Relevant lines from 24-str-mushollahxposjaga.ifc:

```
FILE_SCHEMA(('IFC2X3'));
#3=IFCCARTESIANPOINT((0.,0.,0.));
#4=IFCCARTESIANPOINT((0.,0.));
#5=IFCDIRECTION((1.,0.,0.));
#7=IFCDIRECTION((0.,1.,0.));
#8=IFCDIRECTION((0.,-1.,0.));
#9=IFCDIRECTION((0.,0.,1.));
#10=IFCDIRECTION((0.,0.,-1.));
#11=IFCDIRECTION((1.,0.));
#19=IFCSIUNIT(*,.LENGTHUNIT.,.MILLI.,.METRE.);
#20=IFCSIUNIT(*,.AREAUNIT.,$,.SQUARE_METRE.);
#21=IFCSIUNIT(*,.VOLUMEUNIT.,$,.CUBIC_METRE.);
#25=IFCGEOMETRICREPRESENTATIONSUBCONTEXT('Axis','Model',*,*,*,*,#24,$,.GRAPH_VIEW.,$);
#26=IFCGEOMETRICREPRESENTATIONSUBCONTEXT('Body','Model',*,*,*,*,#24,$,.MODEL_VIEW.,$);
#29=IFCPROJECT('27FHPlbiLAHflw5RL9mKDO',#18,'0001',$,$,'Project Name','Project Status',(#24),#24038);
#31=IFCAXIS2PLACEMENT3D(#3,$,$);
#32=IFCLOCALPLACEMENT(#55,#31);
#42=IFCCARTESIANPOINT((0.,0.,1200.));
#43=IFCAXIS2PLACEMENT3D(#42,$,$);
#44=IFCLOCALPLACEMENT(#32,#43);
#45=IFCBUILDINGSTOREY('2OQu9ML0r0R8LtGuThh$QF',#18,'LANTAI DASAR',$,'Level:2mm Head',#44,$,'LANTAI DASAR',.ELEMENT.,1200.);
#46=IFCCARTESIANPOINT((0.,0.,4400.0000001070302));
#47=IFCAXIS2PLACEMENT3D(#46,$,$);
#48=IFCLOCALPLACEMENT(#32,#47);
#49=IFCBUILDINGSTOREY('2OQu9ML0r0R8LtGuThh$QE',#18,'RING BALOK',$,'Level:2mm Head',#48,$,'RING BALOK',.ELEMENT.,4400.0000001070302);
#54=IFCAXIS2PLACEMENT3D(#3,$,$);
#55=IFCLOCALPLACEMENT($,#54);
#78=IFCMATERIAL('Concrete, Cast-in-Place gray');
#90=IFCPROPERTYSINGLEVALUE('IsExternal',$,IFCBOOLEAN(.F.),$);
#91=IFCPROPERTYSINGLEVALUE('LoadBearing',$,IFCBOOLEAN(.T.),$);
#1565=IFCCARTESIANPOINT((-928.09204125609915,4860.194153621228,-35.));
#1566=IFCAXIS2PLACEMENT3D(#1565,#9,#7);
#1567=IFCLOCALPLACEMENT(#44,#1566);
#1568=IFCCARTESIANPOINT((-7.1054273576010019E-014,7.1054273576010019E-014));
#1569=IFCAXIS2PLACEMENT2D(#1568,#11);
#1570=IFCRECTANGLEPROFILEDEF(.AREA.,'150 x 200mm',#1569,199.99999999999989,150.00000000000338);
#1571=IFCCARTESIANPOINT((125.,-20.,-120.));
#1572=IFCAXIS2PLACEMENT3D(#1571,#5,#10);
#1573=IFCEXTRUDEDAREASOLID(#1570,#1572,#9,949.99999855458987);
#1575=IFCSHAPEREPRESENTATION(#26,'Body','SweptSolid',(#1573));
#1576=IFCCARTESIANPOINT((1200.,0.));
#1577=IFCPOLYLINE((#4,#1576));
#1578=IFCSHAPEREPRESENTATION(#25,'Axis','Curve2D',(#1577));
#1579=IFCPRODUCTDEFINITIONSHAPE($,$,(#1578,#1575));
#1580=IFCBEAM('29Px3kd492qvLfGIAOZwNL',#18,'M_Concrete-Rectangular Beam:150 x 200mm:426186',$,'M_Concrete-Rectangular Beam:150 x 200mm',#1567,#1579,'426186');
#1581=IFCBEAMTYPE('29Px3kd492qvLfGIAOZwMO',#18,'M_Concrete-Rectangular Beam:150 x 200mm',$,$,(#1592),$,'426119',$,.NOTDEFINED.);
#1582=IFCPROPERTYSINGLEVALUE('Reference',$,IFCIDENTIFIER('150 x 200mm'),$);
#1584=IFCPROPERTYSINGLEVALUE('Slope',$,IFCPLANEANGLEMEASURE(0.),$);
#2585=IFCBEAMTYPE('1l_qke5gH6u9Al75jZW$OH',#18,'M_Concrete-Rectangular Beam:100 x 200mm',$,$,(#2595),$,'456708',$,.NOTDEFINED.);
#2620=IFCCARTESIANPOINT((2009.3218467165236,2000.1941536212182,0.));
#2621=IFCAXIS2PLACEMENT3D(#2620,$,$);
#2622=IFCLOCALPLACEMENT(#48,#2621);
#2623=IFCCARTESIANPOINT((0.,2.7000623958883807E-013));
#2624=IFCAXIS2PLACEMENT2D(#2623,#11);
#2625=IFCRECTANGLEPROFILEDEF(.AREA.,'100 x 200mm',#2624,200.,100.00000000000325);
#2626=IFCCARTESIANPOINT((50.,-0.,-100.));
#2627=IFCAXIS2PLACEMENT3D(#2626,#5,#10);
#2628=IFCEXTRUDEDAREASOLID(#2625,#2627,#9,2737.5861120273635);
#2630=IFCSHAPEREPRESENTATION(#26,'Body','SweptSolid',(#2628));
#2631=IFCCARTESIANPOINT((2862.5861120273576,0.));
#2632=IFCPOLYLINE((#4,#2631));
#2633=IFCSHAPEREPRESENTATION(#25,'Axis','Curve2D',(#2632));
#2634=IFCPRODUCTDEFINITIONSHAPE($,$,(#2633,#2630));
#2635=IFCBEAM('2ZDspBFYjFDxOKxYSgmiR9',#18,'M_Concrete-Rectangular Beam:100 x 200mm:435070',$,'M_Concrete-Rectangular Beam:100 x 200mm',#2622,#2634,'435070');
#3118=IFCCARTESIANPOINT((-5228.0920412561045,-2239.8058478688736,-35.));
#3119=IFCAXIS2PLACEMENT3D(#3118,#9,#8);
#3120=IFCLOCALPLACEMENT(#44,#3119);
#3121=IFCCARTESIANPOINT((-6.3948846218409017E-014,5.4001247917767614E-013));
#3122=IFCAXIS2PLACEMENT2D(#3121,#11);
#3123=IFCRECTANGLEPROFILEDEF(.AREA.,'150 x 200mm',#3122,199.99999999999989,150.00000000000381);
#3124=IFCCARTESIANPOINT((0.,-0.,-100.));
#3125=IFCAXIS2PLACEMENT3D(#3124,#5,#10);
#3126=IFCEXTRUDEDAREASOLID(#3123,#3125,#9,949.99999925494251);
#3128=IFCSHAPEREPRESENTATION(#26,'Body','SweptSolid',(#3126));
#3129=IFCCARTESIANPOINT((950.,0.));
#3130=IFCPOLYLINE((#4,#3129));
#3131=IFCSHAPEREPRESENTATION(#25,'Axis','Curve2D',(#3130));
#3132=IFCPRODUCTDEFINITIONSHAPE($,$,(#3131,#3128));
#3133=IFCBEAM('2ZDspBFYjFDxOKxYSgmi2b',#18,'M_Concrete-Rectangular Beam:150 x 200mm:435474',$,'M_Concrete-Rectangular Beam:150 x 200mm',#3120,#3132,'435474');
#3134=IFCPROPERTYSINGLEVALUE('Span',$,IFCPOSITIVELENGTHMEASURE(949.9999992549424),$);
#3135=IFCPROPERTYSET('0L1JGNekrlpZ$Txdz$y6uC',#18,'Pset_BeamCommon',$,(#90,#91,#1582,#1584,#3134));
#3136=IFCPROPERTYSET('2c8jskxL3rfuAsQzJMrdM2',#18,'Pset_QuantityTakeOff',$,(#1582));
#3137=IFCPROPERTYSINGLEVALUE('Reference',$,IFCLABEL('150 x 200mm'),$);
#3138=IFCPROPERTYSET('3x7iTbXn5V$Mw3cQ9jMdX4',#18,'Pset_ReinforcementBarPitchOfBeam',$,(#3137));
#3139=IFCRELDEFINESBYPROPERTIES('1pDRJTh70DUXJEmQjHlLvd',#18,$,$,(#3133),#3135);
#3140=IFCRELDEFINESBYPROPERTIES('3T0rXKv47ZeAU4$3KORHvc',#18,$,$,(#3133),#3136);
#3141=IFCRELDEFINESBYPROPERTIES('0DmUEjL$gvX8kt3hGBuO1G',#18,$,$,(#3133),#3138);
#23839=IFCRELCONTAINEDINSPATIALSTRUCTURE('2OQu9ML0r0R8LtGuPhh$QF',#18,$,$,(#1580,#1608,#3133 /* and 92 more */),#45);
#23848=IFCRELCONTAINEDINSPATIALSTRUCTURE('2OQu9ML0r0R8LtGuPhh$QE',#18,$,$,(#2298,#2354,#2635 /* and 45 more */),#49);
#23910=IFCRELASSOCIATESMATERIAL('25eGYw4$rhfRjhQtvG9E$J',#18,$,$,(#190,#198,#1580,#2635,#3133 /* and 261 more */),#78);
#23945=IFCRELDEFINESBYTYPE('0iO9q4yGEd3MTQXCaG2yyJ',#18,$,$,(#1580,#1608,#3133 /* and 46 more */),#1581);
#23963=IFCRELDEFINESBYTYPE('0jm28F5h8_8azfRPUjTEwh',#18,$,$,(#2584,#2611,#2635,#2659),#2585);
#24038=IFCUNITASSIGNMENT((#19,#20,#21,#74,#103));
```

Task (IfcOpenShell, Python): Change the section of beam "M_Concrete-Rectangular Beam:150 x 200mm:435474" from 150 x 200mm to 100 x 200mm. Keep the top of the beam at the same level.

```python
import ifcopenshell
import ifcopenshell.api.pset
import ifcopenshell.api.type
import ifcopenshell.util.element
import ifcopenshell.util.representation

model = ifcopenshell.open("24-str-mushollahxposjaga.ifc")

member = model.by_guid("2ZDspBFYjFDxOKxYSgmi2b")
source = next(p for p in model.by_type("IfcRectangleProfileDef") if p.ProfileName == "100 x 200mm")

body = ifcopenshell.util.representation.get_representation(member, "Model", "Body")
solid = body.Items[0]
old_profile = solid.SweptArea

# Copy the section's sizes but keep this member's own profile position.
profile = ifcopenshell.util.element.copy(model, source)
# Profiles are centred, so shift by half the change in depth to hold the top.
shift = (old_profile.XDim - profile.XDim) / 2
x, y = old_profile.Position.Location.Coordinates
up = (-1.0, 0.0)  # upwards, in the solid's own plane
location = model.createIfcCartesianPoint((x + up[0] * shift, y + up[1] * shift))
profile.Position = model.createIfcAxis2Placement2D(location, old_profile.Position.RefDirection)
solid.SweptArea = profile
if not model.get_total_inverses(old_profile):
    ifcopenshell.util.element.remove_deep2(model, old_profile)

new_type = model.by_id(2585)
ifcopenshell.api.type.assign_type(
    model, related_objects=[member], relating_type=new_type, should_map_representations=False
)
member.Name = member.Name.replace("150 x 200mm", "100 x 200mm")
member.ObjectType = "M_Concrete-Rectangular Beam:100 x 200mm"
pset = model.by_id(ifcopenshell.util.element.get_pset(member, "Pset_BeamCommon", should_inherit=False)["id"])
ifcopenshell.api.pset.edit_pset(model, pset=pset, properties={"Reference": "100 x 200mm"})
pset = model.by_id(ifcopenshell.util.element.get_pset(member, "Pset_QuantityTakeOff", should_inherit=False)["id"])
ifcopenshell.api.pset.edit_pset(model, pset=pset, properties={"Reference": "100 x 200mm"})
pset = model.by_id(ifcopenshell.util.element.get_pset(member, "Pset_ReinforcementBarPitchOfBeam", should_inherit=False)["id"])
ifcopenshell.api.pset.edit_pset(model, pset=pset, properties={"Reference": "100 x 200mm"})

print(solid.SweptArea)

model.write("24-str-mushollahxposjaga_edited.ifc")
```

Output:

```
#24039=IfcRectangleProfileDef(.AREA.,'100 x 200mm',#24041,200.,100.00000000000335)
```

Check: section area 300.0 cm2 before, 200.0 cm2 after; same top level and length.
